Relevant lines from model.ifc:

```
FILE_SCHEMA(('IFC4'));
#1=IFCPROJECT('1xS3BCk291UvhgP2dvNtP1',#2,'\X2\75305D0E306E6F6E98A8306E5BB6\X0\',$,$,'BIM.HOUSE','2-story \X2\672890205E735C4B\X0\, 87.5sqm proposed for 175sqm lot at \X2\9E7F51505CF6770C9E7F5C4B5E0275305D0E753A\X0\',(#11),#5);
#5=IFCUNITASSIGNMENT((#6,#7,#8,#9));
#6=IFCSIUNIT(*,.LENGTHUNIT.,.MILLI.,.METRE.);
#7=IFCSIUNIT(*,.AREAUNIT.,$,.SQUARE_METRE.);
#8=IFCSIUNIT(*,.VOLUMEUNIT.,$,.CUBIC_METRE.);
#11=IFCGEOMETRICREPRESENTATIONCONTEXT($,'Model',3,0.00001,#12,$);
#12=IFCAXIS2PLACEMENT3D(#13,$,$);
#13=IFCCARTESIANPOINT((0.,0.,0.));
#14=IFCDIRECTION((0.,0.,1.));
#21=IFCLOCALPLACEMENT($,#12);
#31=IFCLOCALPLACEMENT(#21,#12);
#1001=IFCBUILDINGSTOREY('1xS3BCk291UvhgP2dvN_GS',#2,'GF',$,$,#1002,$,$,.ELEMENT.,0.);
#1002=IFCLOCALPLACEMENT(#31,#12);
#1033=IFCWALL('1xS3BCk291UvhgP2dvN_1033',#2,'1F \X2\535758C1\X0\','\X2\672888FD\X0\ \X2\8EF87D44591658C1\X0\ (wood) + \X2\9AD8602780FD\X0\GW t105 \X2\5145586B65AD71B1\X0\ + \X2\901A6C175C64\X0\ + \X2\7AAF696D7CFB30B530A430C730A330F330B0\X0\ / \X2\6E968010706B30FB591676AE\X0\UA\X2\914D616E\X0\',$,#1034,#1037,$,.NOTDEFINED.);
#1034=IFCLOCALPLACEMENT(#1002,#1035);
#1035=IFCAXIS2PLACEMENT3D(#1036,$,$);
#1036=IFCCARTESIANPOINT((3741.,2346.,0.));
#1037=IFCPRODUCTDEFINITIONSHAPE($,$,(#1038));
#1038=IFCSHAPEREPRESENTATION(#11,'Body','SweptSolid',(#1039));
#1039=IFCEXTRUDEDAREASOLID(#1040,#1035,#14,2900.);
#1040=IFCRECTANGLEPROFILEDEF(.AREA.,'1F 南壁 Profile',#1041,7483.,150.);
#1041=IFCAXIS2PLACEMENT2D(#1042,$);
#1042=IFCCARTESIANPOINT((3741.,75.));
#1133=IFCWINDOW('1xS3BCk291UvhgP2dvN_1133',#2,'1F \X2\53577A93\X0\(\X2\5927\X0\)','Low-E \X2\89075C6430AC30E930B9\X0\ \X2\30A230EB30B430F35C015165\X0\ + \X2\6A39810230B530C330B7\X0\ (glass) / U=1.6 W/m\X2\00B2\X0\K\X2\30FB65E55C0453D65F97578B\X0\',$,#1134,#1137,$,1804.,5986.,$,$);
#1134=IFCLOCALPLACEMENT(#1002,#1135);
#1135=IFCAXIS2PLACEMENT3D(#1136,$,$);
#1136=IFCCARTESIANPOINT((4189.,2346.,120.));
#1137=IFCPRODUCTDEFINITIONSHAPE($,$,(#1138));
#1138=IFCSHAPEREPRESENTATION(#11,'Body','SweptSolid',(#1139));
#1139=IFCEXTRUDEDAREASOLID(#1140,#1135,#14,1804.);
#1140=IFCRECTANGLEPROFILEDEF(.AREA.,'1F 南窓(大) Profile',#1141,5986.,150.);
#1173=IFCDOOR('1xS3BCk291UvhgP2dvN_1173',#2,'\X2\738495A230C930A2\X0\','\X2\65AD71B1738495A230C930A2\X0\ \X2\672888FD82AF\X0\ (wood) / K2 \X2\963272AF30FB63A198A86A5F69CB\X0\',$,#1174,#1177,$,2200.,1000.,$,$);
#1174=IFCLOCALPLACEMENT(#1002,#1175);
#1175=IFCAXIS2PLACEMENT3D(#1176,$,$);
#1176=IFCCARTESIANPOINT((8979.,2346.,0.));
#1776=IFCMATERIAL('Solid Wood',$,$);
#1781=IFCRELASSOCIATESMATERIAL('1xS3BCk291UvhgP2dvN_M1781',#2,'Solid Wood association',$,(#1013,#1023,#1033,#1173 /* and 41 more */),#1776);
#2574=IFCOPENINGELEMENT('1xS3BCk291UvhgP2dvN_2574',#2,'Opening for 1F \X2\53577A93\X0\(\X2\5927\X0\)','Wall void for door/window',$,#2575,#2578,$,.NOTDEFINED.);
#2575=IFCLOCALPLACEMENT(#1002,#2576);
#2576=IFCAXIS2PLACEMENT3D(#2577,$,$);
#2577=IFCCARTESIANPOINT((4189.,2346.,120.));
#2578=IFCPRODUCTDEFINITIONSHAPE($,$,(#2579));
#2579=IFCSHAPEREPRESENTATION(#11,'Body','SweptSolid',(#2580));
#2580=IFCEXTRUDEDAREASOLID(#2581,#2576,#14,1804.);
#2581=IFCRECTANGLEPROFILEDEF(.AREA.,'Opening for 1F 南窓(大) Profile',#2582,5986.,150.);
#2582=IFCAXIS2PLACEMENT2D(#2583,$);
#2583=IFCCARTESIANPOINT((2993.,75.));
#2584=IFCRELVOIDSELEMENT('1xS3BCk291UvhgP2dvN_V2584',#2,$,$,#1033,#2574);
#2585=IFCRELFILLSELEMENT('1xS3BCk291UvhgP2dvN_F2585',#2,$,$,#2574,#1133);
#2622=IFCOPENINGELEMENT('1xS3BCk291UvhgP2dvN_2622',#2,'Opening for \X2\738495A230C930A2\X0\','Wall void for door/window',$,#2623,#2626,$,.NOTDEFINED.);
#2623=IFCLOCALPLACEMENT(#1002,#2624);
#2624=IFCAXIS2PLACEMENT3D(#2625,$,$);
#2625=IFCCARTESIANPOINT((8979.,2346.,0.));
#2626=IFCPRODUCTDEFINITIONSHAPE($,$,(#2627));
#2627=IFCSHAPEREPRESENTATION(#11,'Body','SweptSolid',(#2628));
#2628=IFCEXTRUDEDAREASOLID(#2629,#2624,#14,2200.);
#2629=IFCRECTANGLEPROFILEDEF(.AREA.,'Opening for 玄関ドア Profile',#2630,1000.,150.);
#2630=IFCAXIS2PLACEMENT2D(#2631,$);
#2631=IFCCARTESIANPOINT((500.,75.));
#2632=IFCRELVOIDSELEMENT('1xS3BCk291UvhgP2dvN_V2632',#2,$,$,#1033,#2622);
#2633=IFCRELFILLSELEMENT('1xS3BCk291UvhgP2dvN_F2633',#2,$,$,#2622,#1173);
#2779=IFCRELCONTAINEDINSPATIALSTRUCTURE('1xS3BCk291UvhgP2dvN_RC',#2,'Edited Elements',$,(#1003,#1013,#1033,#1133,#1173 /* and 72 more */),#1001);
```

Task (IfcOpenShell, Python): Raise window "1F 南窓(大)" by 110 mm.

```python
import numpy as np
import ifcopenshell
import ifcopenshell.api.geometry
import ifcopenshell.util.placement
import ifcopenshell.util.unit

model = ifcopenshell.open("model.ifc")
unit_scale = ifcopenshell.util.unit.calculate_unit_scale(model)

window = model.by_guid("1xS3BCk291UvhgP2dvN_1133")
opening = window.FillsVoids[0].RelatingOpeningElement
dz = 110.0

shift = np.array([0.0, 0.0, dz])
# The window is not placed relative to its opening, so move both.
for product in (opening, window):
    matrix = ifcopenshell.util.placement.get_local_placement(product.ObjectPlacement)
    matrix[:3, 3] += shift
    ifcopenshell.api.geometry.edit_object_placement(model, product=product, matrix=matrix, is_si=False)

print(f"moved by {dz * unit_scale:+.3f} m")

model.write("model_rev.ifc")
```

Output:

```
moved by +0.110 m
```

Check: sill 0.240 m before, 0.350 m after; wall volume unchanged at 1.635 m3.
